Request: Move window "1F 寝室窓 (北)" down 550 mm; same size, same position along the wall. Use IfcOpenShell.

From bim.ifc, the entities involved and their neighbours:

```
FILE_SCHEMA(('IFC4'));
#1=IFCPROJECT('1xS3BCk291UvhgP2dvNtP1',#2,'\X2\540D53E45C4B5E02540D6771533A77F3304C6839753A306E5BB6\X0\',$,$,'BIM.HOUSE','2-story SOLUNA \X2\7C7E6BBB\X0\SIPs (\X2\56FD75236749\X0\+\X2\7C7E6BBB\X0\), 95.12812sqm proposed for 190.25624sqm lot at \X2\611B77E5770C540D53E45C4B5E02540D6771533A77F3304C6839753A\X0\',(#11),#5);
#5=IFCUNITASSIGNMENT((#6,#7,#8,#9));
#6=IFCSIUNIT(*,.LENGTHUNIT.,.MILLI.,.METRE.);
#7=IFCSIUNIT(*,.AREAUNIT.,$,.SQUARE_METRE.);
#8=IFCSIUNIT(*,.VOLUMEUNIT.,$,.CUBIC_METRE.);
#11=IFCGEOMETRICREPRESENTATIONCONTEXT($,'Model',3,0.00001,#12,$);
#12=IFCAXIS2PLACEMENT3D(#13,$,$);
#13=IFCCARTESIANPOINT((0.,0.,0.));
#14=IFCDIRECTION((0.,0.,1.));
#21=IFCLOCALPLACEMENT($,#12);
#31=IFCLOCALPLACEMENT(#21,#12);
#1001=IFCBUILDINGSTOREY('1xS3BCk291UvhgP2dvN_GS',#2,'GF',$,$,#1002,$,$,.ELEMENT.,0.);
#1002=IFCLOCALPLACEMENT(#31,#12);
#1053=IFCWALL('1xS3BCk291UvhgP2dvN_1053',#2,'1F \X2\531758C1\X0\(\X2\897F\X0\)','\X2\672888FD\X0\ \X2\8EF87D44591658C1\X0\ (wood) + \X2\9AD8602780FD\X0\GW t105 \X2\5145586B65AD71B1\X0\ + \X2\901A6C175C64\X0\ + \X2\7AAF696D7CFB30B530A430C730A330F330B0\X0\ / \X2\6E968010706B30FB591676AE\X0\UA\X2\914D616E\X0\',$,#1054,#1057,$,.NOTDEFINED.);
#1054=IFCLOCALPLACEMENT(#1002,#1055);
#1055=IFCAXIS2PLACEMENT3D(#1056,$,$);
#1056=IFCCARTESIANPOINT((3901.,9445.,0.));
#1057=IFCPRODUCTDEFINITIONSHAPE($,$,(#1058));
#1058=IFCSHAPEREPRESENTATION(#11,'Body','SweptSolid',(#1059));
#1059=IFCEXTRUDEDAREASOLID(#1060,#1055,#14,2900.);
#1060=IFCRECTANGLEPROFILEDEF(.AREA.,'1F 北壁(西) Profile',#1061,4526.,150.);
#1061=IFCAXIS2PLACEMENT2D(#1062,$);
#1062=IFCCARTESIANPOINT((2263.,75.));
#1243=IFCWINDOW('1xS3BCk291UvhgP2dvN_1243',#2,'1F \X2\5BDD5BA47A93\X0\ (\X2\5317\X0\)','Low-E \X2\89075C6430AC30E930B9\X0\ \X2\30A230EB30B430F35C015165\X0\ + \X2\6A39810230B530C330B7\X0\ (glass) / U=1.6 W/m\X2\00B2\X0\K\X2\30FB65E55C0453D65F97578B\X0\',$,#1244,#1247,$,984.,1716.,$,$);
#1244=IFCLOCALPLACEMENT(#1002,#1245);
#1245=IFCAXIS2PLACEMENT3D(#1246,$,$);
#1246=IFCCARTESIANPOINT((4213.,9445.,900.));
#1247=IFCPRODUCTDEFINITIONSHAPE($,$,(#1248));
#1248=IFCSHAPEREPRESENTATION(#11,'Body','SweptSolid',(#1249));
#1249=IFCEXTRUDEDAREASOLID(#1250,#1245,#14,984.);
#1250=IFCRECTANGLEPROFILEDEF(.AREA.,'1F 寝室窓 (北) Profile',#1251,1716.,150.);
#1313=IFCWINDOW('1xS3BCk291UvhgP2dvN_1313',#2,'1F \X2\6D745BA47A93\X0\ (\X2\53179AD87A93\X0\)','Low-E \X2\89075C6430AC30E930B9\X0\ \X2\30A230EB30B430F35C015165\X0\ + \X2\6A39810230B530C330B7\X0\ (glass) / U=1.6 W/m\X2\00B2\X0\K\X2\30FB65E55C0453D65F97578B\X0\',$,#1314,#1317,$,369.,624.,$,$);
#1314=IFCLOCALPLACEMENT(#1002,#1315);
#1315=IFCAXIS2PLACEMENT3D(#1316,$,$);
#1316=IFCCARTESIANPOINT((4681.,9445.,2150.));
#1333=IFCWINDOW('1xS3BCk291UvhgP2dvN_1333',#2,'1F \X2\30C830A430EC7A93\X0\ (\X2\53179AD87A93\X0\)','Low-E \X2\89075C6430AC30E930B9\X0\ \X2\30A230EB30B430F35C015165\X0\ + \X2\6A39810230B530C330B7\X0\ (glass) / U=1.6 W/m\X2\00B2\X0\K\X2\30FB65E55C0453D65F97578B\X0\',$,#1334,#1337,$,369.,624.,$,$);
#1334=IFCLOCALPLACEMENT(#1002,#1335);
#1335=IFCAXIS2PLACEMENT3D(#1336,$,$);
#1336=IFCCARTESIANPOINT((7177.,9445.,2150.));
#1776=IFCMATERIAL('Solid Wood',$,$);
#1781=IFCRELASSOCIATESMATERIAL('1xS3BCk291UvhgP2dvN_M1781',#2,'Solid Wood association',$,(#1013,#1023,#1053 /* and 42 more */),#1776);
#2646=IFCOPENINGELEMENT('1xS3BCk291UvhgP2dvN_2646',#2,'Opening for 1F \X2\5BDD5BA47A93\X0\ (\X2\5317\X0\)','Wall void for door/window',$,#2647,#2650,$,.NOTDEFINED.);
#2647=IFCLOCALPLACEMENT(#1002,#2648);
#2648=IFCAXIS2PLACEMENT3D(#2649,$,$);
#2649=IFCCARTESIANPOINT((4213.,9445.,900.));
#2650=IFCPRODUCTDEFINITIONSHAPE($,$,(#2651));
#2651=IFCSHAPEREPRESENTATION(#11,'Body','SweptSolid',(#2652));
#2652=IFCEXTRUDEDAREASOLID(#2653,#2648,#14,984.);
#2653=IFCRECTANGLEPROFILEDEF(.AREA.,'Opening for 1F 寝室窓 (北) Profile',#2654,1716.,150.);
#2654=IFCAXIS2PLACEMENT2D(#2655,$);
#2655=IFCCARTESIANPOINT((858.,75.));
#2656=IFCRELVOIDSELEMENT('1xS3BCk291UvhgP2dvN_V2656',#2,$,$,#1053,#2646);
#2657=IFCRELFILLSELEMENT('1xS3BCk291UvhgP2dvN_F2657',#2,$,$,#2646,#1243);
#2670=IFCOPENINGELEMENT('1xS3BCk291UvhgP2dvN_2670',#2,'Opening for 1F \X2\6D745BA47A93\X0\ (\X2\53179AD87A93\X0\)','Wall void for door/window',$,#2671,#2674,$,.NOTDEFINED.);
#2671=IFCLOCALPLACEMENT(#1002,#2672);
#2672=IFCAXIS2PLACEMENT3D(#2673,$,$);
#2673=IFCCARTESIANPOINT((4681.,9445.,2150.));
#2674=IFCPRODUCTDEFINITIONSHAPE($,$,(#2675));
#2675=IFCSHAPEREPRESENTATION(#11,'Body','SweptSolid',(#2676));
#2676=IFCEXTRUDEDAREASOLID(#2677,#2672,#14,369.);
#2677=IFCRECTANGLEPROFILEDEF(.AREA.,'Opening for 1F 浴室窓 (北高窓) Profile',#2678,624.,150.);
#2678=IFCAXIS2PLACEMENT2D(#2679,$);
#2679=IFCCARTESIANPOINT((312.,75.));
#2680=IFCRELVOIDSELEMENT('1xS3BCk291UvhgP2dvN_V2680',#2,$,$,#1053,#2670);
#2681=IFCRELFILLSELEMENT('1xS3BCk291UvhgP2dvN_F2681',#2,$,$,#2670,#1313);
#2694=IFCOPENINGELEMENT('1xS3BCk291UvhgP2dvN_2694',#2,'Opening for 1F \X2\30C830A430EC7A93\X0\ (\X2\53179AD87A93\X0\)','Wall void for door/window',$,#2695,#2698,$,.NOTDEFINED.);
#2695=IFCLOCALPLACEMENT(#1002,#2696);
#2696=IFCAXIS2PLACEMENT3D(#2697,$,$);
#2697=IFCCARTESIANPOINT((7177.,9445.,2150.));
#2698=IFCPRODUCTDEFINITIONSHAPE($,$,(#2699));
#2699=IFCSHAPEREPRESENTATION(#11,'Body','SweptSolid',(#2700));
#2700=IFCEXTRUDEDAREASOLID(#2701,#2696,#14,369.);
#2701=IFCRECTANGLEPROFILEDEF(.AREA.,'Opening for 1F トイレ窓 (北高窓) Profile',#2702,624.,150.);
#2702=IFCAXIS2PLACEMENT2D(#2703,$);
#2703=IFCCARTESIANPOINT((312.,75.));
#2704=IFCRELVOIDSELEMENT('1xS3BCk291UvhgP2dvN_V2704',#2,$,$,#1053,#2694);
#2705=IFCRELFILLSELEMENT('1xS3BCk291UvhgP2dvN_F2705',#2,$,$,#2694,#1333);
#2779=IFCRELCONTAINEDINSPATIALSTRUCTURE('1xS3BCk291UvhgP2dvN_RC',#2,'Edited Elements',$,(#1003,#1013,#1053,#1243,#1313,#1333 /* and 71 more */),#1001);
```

```python
import numpy as np
import ifcopenshell
import ifcopenshell.api.geometry
import ifcopenshell.util.placement
import ifcopenshell.util.unit

model = ifcopenshell.open("bim.ifc")
unit_scale = ifcopenshell.util.unit.calculate_unit_scale(model)

window = model.by_guid("1xS3BCk291UvhgP2dvN_1243")
opening = window.FillsVoids[0].RelatingOpeningElement
dz = -0.55 / unit_scale

shift = np.array([0.0, 0.0, dz])
# The window is not placed relative to its opening, so move both.
for product in (opening, window):
    matrix = ifcopenshell.util.placement.get_local_placement(product.ObjectPlacement)
    matrix[:3, 3] += shift
    ifcopenshell.api.geometry.edit_object_placement(model, product=product, matrix=matrix, is_si=False)

print(f"moved by {dz * unit_scale:+.3f} m")

model.write("bim-out.ifc")
```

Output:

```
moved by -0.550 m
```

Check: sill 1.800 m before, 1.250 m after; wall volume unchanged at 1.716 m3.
